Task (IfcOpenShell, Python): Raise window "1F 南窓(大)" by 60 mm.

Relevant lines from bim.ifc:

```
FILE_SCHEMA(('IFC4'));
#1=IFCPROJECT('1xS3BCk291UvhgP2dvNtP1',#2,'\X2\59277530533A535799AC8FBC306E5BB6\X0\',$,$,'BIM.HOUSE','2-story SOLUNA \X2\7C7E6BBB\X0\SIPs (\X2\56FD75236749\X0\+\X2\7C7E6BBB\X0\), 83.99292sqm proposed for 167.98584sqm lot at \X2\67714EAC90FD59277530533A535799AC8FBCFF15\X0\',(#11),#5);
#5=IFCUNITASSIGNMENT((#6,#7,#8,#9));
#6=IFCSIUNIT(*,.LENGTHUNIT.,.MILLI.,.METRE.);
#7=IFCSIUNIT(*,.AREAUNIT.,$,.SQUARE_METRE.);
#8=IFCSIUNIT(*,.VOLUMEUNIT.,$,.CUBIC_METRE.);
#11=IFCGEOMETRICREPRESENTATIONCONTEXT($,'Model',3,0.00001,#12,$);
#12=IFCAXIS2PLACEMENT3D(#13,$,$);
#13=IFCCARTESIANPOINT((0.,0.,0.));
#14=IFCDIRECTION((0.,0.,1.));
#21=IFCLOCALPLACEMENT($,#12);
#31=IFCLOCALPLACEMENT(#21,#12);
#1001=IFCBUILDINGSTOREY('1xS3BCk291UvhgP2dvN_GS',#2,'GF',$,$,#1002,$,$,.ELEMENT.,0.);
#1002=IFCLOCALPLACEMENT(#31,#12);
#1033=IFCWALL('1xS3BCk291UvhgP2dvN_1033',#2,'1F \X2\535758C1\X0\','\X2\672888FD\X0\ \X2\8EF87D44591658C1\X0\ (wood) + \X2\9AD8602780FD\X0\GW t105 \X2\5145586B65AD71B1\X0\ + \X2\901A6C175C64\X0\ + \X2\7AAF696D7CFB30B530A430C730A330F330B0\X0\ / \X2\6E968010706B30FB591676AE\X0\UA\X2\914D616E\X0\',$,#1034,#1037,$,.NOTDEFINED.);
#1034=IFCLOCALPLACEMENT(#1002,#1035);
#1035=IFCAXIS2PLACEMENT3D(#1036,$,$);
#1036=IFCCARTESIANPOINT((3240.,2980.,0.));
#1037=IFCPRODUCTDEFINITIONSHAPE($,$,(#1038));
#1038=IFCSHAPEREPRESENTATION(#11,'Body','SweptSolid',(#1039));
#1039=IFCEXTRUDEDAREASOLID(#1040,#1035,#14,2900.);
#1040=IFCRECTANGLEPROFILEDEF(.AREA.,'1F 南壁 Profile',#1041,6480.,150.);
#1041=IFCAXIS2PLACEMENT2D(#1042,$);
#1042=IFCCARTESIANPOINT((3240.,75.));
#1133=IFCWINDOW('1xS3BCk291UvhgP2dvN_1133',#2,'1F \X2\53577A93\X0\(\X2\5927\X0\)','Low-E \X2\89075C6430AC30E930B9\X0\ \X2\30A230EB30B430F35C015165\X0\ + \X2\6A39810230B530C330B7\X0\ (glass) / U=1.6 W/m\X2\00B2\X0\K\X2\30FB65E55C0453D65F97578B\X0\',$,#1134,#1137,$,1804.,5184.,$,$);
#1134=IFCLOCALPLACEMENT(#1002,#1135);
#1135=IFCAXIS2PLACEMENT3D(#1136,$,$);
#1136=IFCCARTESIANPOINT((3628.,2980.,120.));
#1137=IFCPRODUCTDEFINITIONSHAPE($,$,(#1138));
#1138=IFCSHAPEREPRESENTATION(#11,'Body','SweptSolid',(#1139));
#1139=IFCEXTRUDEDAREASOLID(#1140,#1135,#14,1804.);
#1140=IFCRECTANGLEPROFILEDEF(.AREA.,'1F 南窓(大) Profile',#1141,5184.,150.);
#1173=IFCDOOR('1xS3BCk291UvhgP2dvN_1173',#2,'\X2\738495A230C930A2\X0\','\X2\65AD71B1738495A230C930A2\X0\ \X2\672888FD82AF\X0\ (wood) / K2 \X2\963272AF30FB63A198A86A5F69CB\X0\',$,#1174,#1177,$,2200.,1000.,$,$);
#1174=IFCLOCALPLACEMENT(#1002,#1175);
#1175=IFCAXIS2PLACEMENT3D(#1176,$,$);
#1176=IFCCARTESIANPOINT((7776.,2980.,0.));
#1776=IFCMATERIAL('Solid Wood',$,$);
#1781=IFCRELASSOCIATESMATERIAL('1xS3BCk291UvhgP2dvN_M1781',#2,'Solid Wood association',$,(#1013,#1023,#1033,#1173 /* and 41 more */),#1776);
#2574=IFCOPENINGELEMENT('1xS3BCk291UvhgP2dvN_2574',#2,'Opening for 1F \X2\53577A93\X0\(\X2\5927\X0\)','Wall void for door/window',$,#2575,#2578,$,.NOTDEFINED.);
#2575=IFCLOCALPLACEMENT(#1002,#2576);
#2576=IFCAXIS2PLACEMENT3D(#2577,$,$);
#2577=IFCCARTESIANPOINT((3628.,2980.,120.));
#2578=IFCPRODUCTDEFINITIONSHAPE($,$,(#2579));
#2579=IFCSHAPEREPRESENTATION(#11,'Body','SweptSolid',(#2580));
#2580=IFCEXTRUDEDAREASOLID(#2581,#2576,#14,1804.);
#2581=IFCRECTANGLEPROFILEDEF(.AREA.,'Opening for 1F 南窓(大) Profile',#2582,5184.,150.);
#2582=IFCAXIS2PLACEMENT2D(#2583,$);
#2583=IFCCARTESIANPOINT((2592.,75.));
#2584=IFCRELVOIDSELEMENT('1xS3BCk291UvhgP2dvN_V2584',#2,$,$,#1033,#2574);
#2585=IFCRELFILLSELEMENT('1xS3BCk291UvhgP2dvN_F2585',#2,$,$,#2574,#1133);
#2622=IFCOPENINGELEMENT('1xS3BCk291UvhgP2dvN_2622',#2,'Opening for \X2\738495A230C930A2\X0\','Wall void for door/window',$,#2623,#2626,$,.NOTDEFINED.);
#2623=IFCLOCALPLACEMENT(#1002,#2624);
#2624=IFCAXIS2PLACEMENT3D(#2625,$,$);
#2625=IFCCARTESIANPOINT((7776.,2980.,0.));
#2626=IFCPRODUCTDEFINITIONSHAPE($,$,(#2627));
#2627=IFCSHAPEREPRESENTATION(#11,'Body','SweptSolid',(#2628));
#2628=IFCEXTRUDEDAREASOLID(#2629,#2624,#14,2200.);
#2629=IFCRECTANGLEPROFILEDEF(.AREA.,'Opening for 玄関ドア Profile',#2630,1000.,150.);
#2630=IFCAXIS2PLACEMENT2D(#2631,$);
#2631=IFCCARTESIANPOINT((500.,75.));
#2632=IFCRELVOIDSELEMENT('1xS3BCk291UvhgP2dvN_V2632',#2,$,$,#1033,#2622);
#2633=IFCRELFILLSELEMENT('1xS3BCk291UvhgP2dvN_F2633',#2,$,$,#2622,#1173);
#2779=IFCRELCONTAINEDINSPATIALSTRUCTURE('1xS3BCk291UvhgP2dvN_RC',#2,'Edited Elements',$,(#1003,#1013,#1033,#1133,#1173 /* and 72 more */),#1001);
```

```python
import numpy as np
import ifcopenshell
import ifcopenshell.api.geometry
import ifcopenshell.util.placement
import ifcopenshell.util.unit

model = ifcopenshell.open("bim.ifc")
unit_scale = ifcopenshell.util.unit.calculate_unit_scale(model)

window = model.by_guid("1xS3BCk291UvhgP2dvN_1133")
opening = window.FillsVoids[0].RelatingOpeningElement
dz = 0.06 / unit_scale

shift = np.array([0.0, 0.0, dz])
# The window is not placed relative to its opening, so move both.
for product in (opening, window):
    matrix = ifcopenshell.util.placement.get_local_placement(product.ObjectPlacement)
    matrix[:3, 3] += shift
    ifcopenshell.api.geometry.edit_object_placement(model, product=product, matrix=matrix, is_si=False)

print(f"moved by {dz * unit_scale:+.3f} m")

model.write("bim-out.ifc")
```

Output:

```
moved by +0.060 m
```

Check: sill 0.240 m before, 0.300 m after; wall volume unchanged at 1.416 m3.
